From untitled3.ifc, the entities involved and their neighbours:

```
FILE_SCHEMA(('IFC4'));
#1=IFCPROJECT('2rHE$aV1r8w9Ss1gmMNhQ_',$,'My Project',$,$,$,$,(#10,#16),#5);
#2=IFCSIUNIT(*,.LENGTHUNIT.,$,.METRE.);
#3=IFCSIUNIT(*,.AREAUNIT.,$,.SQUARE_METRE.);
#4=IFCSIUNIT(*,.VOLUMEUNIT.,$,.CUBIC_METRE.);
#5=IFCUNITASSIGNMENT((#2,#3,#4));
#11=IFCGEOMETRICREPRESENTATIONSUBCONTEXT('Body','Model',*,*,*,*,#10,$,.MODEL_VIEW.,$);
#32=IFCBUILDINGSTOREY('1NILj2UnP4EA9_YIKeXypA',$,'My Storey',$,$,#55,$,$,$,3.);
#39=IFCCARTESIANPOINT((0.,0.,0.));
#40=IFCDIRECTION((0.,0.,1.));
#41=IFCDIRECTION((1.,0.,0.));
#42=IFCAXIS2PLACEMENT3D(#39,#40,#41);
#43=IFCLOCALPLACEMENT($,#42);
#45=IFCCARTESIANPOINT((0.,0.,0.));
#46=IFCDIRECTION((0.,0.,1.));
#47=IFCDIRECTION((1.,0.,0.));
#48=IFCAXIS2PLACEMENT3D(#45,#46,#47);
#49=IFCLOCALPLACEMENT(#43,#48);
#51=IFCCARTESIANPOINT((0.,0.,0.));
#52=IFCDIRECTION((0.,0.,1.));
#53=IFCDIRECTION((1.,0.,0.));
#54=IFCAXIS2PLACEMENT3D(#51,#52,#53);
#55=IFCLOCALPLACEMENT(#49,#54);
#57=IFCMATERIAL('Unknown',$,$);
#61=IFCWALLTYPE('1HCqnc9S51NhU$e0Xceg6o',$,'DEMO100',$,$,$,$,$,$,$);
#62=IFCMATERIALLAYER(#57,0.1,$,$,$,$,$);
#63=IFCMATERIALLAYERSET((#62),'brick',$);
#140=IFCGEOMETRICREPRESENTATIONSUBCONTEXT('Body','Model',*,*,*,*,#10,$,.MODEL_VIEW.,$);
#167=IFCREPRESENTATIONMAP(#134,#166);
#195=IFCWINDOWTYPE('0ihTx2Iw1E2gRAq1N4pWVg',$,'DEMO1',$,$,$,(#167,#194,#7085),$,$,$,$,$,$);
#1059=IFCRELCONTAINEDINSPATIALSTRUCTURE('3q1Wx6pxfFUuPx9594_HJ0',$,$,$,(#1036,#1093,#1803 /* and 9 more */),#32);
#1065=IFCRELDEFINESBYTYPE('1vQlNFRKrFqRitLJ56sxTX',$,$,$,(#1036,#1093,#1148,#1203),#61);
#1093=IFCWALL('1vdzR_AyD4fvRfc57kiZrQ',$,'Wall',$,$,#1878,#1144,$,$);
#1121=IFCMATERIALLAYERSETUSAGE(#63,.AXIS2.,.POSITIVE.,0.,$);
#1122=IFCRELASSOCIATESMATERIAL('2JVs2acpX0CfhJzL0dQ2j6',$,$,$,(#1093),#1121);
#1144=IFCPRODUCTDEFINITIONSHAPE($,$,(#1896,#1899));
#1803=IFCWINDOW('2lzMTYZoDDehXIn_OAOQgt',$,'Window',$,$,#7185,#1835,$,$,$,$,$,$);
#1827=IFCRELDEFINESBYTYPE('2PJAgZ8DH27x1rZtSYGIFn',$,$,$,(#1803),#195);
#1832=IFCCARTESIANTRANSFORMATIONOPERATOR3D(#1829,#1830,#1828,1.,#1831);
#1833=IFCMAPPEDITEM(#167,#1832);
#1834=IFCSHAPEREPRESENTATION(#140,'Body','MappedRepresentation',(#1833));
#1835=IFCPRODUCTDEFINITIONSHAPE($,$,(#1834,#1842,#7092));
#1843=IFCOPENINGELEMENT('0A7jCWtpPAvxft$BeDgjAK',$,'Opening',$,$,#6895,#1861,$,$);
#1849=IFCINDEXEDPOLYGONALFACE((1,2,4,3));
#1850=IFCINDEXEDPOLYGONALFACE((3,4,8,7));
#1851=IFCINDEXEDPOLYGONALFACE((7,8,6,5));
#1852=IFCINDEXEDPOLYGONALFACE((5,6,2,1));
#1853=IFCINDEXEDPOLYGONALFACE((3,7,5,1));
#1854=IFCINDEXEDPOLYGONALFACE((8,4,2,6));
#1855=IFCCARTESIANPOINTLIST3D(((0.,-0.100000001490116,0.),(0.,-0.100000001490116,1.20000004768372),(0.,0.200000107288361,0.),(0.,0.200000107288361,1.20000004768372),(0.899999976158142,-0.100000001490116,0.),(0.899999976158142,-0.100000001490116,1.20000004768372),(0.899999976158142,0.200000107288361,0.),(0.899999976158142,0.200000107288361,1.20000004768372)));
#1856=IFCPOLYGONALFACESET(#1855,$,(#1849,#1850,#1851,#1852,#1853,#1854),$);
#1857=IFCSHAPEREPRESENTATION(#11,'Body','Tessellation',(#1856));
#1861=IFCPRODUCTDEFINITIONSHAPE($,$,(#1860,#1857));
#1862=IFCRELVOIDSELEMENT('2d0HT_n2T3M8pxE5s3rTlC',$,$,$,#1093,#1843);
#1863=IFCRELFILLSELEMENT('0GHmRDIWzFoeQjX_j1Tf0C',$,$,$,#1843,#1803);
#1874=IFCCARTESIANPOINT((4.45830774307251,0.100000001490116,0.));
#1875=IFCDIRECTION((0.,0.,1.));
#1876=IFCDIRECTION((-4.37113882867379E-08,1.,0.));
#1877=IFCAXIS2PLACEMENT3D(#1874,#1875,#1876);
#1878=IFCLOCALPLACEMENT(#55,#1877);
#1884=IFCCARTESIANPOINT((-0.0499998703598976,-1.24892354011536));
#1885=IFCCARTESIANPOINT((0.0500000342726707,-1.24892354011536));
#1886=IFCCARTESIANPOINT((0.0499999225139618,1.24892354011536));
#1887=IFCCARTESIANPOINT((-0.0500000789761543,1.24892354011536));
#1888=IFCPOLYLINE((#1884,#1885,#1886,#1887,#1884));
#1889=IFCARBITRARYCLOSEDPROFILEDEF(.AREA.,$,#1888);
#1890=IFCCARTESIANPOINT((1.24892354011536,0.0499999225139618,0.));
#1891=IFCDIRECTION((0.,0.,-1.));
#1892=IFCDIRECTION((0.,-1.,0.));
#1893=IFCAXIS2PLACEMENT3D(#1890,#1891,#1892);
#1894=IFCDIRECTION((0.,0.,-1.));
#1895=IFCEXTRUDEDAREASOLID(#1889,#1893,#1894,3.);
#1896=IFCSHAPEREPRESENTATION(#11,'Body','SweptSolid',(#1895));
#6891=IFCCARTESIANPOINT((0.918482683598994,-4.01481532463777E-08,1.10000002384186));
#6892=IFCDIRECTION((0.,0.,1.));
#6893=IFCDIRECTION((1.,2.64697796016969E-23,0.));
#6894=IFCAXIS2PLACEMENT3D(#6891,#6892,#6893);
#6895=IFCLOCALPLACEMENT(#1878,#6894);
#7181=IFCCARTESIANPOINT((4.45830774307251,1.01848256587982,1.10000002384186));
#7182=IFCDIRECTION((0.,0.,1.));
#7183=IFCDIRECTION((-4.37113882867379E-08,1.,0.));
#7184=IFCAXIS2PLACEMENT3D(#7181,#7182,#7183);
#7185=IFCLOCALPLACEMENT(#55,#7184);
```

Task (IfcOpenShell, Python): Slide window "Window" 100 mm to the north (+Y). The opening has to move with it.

```python
import ifcopenshell
import ifcopenshell.api.geometry
import ifcopenshell.util.placement
import ifcopenshell.util.unit

model = ifcopenshell.open("untitled3.ifc")
unit_scale = ifcopenshell.util.unit.calculate_unit_scale(model)

window = model.by_guid("2lzMTYZoDDehXIn_OAOQgt")
opening = window.FillsVoids[0].RelatingOpeningElement
wall = opening.VoidsElements[0].RelatingBuildingElement

wall_matrix = ifcopenshell.util.placement.get_local_placement(wall.ObjectPlacement)
shift = wall_matrix[:3, 0] * 0.1 / unit_scale
before = ifcopenshell.util.placement.get_local_placement(window.ObjectPlacement)[:3, 3].copy()

# The window is not placed relative to its opening, so move both.
for product in (opening, window):
    matrix = ifcopenshell.util.placement.get_local_placement(product.ObjectPlacement)
    matrix[:3, 3] += shift
    ifcopenshell.api.geometry.edit_object_placement(model, product=product, matrix=matrix, is_si=False)

after = ifcopenshell.util.placement.get_local_placement(window.ObjectPlacement)[:3, 3]
print("window moved by", (after - before).round(3) + 0.0)

model.write("untitled3_v2.ifc")
```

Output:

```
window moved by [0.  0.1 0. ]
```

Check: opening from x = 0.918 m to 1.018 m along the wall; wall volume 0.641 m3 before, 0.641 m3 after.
